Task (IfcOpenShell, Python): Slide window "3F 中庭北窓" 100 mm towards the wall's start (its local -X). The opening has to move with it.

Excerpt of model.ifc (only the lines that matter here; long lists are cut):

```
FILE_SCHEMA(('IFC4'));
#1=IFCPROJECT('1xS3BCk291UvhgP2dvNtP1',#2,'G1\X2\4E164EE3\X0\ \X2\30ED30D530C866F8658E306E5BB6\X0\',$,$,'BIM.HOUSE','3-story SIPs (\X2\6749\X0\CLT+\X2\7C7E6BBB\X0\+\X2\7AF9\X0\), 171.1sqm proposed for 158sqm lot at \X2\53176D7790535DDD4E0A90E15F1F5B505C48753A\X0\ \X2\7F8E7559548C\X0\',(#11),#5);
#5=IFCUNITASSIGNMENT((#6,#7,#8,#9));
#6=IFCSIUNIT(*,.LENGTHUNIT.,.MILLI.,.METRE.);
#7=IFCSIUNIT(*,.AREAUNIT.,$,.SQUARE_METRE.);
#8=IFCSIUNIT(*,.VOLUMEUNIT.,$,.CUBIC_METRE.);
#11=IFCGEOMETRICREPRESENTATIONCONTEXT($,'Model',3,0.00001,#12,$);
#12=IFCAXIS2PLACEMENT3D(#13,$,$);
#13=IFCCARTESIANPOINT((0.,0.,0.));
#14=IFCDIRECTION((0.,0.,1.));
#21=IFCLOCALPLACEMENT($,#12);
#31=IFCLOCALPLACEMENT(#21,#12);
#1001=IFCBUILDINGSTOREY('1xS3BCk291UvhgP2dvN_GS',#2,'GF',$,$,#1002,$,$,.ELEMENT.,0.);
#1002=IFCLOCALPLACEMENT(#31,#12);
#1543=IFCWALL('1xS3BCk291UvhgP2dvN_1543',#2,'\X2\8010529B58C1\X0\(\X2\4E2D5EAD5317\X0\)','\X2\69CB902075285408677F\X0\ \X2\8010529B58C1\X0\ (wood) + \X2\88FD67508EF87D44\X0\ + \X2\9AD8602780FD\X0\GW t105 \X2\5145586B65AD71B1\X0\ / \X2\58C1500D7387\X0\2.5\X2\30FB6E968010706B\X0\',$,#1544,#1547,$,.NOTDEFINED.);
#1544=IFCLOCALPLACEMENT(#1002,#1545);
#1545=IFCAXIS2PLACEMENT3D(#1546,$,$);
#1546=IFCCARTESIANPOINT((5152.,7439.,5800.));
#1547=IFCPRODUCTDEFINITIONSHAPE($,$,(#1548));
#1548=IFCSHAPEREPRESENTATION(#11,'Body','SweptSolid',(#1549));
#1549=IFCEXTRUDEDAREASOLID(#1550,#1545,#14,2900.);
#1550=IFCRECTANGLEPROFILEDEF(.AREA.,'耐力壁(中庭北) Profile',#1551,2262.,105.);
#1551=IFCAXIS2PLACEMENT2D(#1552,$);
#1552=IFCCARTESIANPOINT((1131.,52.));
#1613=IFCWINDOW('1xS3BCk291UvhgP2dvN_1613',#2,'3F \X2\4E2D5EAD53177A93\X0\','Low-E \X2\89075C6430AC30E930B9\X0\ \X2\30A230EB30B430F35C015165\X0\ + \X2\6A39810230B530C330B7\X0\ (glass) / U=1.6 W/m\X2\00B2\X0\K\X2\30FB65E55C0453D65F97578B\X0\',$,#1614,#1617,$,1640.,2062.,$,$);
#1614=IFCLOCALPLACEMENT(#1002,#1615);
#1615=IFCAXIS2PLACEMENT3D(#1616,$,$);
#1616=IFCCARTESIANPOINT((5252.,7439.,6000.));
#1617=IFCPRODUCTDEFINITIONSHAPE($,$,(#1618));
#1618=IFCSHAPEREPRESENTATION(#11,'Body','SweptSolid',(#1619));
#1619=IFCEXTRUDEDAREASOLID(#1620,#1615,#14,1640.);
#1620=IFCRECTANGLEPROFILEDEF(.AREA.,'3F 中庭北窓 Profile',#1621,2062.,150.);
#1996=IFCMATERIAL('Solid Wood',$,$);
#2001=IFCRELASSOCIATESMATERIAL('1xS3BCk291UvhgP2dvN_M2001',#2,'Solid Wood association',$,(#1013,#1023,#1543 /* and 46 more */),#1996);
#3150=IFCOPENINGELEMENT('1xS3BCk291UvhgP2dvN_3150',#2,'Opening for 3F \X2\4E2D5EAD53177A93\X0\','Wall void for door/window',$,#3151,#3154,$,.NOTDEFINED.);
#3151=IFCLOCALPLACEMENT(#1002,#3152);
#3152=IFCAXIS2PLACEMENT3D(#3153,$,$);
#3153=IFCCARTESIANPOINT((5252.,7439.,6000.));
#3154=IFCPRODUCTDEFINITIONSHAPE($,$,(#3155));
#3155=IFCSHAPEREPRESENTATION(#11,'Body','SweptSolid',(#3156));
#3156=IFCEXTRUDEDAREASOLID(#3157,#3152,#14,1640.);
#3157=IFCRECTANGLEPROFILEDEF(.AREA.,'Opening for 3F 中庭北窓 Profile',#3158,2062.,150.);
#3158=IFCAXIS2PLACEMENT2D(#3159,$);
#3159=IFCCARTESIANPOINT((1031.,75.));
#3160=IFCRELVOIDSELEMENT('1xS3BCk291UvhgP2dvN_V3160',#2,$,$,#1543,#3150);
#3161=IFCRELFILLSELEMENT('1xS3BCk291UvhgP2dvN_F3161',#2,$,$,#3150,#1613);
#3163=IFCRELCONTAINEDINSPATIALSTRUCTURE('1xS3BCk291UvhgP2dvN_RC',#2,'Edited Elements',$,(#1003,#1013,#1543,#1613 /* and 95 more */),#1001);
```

```python
import ifcopenshell
import ifcopenshell.api.geometry
import ifcopenshell.util.placement

model = ifcopenshell.open("model.ifc")

window = model.by_guid("1xS3BCk291UvhgP2dvN_1613")
opening = window.FillsVoids[0].RelatingOpeningElement
wall = opening.VoidsElements[0].RelatingBuildingElement

wall_matrix = ifcopenshell.util.placement.get_local_placement(wall.ObjectPlacement)
shift = wall_matrix[:3, 0] * -100.0
before = ifcopenshell.util.placement.get_local_placement(window.ObjectPlacement)[:3, 3].copy()

# The window is not placed relative to its opening, so move both.
for product in (opening, window):
    matrix = ifcopenshell.util.placement.get_local_placement(product.ObjectPlacement)
    matrix[:3, 3] += shift
    ifcopenshell.api.geometry.edit_object_placement(model, product=product, matrix=matrix, is_si=False)

after = ifcopenshell.util.placement.get_local_placement(window.ObjectPlacement)[:3, 3]
print("window moved by", (after - before).round(3) + 0.0)

model.write("model_rev.ifc")
```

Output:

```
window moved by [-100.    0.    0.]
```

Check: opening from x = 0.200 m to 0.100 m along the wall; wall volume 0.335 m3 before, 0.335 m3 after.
